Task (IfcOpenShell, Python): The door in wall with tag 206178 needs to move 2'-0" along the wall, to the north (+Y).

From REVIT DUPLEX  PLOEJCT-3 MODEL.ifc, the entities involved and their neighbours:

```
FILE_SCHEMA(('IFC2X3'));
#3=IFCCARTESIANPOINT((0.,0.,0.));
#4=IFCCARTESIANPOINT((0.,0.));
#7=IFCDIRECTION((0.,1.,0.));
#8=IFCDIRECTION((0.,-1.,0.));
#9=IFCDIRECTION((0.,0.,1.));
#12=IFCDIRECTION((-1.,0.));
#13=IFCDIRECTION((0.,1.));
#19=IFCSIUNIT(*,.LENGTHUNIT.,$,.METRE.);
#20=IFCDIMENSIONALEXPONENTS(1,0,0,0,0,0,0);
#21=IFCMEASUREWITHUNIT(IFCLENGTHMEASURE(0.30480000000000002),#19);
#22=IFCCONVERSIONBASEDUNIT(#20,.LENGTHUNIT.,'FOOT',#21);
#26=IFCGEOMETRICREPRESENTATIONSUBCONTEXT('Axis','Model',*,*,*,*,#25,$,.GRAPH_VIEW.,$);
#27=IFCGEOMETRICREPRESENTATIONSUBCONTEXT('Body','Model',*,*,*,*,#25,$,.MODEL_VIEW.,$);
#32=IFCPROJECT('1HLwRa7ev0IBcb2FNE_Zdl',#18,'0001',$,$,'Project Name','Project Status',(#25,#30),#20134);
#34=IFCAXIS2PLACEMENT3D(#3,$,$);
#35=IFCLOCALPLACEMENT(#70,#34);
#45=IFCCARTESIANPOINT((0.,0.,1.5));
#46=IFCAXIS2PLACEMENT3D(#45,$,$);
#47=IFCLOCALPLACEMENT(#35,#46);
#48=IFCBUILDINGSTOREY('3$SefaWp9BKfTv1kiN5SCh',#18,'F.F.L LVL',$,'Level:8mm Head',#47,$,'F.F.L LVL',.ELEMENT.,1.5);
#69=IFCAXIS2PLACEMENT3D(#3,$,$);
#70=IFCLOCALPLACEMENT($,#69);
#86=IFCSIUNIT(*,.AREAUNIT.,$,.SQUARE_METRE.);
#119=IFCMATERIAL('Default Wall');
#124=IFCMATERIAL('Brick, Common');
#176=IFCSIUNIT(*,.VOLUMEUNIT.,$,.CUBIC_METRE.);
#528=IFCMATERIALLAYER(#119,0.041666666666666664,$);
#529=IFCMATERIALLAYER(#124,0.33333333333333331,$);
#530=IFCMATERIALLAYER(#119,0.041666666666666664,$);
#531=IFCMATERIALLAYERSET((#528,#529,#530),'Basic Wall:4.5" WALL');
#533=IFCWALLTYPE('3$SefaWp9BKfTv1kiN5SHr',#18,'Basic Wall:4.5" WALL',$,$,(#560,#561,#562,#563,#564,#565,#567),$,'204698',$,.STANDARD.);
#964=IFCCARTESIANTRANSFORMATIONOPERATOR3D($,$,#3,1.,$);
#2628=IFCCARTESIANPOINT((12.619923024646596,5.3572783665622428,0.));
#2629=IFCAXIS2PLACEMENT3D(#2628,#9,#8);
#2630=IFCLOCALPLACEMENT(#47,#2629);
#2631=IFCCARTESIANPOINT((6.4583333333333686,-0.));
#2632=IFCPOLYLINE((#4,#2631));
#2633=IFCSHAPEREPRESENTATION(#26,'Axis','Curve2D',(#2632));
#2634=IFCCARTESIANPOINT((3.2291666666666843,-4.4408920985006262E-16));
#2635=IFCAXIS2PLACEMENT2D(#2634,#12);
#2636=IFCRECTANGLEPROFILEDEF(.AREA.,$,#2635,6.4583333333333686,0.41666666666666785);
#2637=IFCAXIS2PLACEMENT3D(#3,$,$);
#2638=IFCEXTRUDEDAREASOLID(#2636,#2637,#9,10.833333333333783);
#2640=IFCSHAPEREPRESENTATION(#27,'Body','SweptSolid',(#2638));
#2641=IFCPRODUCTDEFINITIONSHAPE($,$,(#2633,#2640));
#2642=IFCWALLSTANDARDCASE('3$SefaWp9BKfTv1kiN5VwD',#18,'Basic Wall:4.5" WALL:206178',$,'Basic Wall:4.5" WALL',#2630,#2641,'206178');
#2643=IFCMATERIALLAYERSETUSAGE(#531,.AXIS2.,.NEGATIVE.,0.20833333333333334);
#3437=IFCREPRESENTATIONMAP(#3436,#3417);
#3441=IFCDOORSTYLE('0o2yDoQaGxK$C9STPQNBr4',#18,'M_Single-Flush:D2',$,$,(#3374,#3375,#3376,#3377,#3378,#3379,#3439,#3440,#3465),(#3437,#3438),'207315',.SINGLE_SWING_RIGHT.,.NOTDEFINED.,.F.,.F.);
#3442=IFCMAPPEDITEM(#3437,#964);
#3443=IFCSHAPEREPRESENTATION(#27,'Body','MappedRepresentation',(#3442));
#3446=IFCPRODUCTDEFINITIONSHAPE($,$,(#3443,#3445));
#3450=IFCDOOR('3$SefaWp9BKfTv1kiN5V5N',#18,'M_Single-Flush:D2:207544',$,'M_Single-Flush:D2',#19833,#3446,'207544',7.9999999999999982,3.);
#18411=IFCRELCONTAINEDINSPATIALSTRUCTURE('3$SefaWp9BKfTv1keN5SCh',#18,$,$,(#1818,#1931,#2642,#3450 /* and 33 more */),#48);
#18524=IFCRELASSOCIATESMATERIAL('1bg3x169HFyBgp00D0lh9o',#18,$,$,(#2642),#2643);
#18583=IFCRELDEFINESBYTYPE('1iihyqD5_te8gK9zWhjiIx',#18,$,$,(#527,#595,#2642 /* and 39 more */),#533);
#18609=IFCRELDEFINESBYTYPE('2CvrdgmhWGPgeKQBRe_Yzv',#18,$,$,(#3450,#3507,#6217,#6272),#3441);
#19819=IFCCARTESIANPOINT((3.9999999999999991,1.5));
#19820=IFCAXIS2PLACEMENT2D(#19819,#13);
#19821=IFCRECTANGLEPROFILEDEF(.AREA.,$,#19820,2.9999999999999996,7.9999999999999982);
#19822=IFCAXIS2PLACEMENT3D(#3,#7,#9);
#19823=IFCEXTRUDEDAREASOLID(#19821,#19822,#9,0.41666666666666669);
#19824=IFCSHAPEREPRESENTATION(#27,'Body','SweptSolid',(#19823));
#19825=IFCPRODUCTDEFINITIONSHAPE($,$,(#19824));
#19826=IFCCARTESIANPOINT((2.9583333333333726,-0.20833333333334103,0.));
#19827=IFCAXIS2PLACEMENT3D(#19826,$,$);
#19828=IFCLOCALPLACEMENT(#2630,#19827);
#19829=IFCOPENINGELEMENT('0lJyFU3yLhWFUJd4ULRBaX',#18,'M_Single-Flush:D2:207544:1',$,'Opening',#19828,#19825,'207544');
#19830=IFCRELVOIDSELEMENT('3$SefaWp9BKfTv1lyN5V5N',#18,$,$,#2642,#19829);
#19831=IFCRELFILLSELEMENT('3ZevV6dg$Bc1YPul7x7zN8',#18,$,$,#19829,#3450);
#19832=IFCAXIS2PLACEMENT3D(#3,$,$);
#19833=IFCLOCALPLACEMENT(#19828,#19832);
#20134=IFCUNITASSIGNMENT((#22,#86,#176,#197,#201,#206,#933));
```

```python
import ifcopenshell
import ifcopenshell.api.geometry
import ifcopenshell.util.placement
import ifcopenshell.util.unit

model = ifcopenshell.open("REVIT DUPLEX  PLOEJCT-3 MODEL.ifc")
unit_scale = ifcopenshell.util.unit.calculate_unit_scale(model)

door = model.by_id(3450)
opening = door.FillsVoids[0].RelatingOpeningElement
wall = opening.VoidsElements[0].RelatingBuildingElement

wall_matrix = ifcopenshell.util.placement.get_local_placement(wall.ObjectPlacement)
shift = wall_matrix[:3, 0] * -24 * 0.0254 / unit_scale
before = ifcopenshell.util.placement.get_local_placement(door.ObjectPlacement)[:3, 3].copy()

# The door is placed relative to its opening, so it follows when the opening moves.
matrix = ifcopenshell.util.placement.get_local_placement(opening.ObjectPlacement)
matrix[:3, 3] += shift
ifcopenshell.api.geometry.edit_object_placement(
    model, product=opening, matrix=matrix, is_si=False, should_transform_children=True
)

after = ifcopenshell.util.placement.get_local_placement(door.ObjectPlacement)[:3, 3]
print("door moved by", (after - before).round(3) + 0.0)

model.write("REVIT DUPLEX  PLOEJCT-3 MODEL_rev.ifc")
```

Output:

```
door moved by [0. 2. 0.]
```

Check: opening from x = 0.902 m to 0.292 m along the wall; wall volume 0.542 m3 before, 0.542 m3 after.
